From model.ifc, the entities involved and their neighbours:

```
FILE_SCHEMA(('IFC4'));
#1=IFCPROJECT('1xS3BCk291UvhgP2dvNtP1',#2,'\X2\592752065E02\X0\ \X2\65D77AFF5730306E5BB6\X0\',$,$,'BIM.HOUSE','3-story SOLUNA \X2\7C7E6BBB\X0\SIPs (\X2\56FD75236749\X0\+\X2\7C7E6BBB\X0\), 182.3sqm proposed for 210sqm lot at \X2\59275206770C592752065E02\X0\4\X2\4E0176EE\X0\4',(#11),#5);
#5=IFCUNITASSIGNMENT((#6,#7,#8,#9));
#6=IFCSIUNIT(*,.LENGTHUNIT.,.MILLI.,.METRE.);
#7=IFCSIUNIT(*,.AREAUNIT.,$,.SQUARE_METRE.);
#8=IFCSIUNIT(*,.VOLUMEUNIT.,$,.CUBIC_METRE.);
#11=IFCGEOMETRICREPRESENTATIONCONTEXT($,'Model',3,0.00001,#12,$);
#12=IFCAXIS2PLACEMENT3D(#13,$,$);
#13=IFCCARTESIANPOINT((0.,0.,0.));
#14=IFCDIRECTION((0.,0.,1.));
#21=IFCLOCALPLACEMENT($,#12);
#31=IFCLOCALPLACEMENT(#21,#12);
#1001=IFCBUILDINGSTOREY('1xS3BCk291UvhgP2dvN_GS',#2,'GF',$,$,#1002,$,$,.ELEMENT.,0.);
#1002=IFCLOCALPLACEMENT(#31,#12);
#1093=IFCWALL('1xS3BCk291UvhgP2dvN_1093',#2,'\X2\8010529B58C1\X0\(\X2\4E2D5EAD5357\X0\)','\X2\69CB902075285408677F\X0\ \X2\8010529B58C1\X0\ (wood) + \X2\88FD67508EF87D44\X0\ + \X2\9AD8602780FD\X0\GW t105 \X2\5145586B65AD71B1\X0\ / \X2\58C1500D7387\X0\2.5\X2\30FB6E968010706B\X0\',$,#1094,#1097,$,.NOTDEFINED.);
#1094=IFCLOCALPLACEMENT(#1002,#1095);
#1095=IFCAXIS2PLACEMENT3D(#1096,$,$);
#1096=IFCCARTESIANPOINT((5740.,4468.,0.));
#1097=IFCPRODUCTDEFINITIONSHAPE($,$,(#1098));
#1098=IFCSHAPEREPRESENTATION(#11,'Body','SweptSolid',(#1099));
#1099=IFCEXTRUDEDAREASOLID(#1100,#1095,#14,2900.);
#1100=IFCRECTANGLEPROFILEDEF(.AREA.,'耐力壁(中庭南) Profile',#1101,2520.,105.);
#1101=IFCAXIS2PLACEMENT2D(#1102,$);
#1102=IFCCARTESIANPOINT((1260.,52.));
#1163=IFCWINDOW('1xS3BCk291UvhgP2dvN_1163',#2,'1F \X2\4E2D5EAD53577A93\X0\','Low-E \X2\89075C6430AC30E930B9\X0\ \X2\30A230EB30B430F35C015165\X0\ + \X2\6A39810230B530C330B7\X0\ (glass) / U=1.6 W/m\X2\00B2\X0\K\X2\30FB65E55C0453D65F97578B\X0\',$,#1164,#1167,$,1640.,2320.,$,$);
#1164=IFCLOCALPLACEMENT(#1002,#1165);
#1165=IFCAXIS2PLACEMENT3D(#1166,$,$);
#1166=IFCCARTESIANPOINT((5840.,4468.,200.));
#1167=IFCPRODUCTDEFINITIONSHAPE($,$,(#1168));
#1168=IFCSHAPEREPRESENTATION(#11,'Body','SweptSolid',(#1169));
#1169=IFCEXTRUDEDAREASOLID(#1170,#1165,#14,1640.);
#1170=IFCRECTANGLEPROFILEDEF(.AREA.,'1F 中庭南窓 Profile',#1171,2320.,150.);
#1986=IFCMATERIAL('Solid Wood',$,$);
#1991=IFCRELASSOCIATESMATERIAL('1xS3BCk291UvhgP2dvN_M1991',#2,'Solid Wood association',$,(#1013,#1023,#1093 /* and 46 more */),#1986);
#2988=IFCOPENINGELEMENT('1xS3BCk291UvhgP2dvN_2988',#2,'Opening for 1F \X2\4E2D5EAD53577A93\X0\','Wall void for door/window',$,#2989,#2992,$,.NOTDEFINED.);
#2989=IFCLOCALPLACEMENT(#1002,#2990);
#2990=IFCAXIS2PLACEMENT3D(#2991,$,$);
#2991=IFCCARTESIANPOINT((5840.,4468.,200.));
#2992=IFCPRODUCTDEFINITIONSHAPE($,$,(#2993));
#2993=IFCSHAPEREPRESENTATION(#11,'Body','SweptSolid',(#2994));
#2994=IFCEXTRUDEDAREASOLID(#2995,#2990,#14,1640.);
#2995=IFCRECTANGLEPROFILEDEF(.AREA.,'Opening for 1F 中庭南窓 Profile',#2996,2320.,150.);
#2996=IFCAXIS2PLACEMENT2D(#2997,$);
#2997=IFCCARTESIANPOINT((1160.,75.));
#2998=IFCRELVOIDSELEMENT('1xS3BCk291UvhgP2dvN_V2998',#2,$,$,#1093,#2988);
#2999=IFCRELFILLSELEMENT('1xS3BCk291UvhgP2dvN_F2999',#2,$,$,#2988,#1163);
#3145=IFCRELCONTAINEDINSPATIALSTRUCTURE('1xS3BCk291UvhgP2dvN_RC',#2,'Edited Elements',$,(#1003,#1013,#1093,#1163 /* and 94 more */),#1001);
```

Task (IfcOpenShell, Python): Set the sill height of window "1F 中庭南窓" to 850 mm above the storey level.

```python
import numpy as np
import ifcopenshell
import ifcopenshell.api.geometry
import ifcopenshell.geom
import ifcopenshell.util.element
import ifcopenshell.util.placement
import ifcopenshell.util.shape
import ifcopenshell.util.unit

model = ifcopenshell.open("model.ifc")
unit_scale = ifcopenshell.util.unit.calculate_unit_scale(model)

window = model.by_id(1163)
opening = window.FillsVoids[0].RelatingOpeningElement
storey = ifcopenshell.util.element.get_container(window, ifc_class="IfcBuildingStorey")
level = ifcopenshell.util.placement.get_local_placement(storey.ObjectPlacement)[2, 3]

# The opening's origin need not be at the sill, so measure its lowest point.
shape = ifcopenshell.geom.create_shape(ifcopenshell.geom.settings(), opening)
bottom = ifcopenshell.util.shape.get_shape_bottom_elevation(shape, shape.geometry) / unit_scale
dz = level + 0.85 / unit_scale - bottom

shift = np.array([0.0, 0.0, dz])
# The window is not placed relative to its opening, so move both.
for product in (opening, window):
    matrix = ifcopenshell.util.placement.get_local_placement(product.ObjectPlacement)
    matrix[:3, 3] += shift
    ifcopenshell.api.geometry.edit_object_placement(model, product=product, matrix=matrix, is_si=False)

print(f"moved by {dz * unit_scale:+.3f} m")

model.write("model_v2.ifc")
```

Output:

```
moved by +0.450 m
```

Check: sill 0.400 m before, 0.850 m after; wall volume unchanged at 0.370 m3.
